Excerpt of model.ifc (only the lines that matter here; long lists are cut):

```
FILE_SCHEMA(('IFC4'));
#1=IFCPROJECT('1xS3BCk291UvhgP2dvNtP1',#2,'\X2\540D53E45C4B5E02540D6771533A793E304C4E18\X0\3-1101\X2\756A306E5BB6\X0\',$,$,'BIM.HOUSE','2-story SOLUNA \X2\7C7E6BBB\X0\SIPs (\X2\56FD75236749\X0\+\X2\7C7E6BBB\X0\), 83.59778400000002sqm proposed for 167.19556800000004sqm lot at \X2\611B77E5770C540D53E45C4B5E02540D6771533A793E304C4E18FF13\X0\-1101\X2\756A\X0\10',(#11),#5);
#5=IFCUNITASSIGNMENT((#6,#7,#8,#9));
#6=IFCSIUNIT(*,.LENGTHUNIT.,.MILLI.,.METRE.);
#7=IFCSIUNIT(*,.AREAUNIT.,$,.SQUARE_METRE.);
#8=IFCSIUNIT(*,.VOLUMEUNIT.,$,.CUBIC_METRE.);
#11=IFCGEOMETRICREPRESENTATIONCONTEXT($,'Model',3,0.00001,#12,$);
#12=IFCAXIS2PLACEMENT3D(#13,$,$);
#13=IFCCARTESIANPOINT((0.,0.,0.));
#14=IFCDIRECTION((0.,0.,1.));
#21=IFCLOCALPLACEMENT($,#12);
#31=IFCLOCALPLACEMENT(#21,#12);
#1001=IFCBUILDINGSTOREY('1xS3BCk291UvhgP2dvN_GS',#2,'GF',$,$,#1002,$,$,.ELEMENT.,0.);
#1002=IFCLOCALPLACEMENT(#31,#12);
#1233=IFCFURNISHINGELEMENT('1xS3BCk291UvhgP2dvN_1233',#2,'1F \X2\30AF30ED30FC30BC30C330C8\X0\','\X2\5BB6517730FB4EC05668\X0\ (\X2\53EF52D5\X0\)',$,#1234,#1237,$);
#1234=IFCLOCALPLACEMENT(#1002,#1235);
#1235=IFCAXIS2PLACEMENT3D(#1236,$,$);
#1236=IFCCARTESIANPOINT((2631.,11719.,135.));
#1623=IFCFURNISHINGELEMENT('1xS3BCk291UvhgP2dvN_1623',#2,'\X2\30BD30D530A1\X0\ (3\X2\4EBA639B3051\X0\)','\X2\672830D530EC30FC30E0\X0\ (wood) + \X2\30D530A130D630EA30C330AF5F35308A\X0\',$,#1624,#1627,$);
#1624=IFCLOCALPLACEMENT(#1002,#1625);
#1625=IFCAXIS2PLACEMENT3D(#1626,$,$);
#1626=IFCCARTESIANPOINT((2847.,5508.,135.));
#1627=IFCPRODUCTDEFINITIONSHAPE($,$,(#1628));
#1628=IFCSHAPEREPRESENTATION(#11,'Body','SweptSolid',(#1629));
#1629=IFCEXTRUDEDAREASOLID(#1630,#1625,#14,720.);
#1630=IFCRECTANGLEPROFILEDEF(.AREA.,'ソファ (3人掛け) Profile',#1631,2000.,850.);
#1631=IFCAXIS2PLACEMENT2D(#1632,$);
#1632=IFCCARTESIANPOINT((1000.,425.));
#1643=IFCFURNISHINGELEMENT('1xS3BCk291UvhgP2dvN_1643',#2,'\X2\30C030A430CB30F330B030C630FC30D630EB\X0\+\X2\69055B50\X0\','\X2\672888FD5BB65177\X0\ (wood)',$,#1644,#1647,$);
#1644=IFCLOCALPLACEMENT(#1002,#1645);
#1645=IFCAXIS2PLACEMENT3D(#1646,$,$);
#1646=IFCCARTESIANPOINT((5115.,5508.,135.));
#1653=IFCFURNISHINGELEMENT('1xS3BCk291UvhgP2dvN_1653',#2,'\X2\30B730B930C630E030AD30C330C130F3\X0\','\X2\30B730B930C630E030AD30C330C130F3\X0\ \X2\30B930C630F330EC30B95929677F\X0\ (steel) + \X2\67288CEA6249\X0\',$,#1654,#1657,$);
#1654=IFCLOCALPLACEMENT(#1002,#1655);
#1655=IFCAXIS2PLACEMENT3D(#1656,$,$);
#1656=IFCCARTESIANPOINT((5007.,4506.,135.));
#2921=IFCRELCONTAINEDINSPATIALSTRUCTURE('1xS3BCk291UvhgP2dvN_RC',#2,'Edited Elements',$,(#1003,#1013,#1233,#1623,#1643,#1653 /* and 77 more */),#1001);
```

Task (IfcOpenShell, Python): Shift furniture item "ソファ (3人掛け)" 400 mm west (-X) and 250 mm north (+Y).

```python
import ifcopenshell
import ifcopenshell.api.geometry
import ifcopenshell.util.placement
import ifcopenshell.util.unit

model = ifcopenshell.open("model.ifc")
unit_scale = ifcopenshell.util.unit.calculate_unit_scale(model)

item = model.by_id(1623)
matrix = ifcopenshell.util.placement.get_local_placement(item.ObjectPlacement)
matrix[0, 3] -= 0.4 / unit_scale
matrix[1, 3] += 0.25 / unit_scale
ifcopenshell.api.geometry.edit_object_placement(model, product=item, matrix=matrix, is_si=False)

print(ifcopenshell.util.placement.get_local_placement(item.ObjectPlacement).round(3) + 0.0)

model.write("model_rev.ifc")
```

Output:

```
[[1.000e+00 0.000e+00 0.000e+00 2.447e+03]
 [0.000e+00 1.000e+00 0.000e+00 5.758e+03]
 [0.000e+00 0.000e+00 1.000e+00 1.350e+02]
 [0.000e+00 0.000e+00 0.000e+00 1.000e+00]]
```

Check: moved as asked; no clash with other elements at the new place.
